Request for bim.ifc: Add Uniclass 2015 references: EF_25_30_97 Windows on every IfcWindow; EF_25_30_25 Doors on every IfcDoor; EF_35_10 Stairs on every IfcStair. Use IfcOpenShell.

First a look at what the model holds.

```python
import ifcopenshell

model = ifcopenshell.open("bim.ifc")
print(model.schema)
print("classifications:", [c.Name for c in model.by_type("IfcClassification")])
for ifc_class in ("IfcDoor", "IfcRoof", "IfcStair", "IfcWall", "IfcWindow"):
    print(ifc_class, len(model.by_type(ifc_class)))
```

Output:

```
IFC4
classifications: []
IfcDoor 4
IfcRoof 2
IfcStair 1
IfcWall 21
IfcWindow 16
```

```python
import ifcopenshell
import ifcopenshell.api.classification

model = ifcopenshell.open("bim.ifc")

system = ifcopenshell.api.classification.add_classification(model, classification="Uniclass 2015")

codes = {
    "IfcWindow": ("EF_25_30_97", "Windows"),
    "IfcDoor": ("EF_25_30_25", "Doors"),
    "IfcStair": ("EF_35_10", "Stairs"),
}
for ifc_class, (code, name) in codes.items():
    products = model.by_type(ifc_class)
    ifcopenshell.api.classification.add_reference(
        model, products=products, classification=system, identification=code, name=name
    )
    print(code, len(products))

model.write("bim-out.ifc")
```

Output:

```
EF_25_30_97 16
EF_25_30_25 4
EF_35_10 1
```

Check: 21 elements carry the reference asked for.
